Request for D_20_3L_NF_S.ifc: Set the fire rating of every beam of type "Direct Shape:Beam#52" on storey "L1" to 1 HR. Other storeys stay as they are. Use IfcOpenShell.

First a look at what the model holds.

```python
import ifcopenshell
import ifcopenshell.util.element

model = ifcopenshell.open("D_20_3L_NF_S.ifc")
print(model.schema)
storey = next(s for s in model.by_type("IfcBuildingStorey") if s.Name == "L1")
beams = [e for e in ifcopenshell.util.element.get_decomposition(storey) if e.is_a("IfcBeam")]
seen = {}
for e in beams:
    element_type = ifcopenshell.util.element.get_type(e)
    key = (element_type.Name if element_type != e and element_type else None, ifcopenshell.util.element.get_pset(e, "Pset_BeamCommon", "FireRating"))
    seen[key] = seen.get(key, 0) + 1
for (name, value), count in sorted(seen.items(), key=str):
    print(count, "x", name, "|", value)
```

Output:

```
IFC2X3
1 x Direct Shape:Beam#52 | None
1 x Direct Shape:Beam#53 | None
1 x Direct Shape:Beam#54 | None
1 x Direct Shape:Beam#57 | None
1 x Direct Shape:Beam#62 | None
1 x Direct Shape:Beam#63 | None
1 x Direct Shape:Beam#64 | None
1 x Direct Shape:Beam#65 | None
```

```python
import ifcopenshell
import ifcopenshell.api.pset
import ifcopenshell.util.element

model = ifcopenshell.open("D_20_3L_NF_S.ifc")

storey = next(s for s in model.by_type("IfcBuildingStorey") if s.Name == "L1")
beams = [e for e in ifcopenshell.util.element.get_decomposition(storey) if e.is_a("IfcBeam")]

count = 0
for e in beams:
    element_type = ifcopenshell.util.element.get_type(e)
    if element_type in (None, e) or element_type.Name != "Direct Shape:Beam#52":
        continue
    # add_pset returns the element's existing set when there is one.
    pset = ifcopenshell.api.pset.add_pset(model, product=e, name="Pset_BeamCommon")
    ifcopenshell.api.pset.edit_pset(model, pset=pset, properties={"FireRating": "1 HR"})
    count += 1

print(count, "beams updated")

model.write("D_20_3L_NF_S_rev.ifc")
```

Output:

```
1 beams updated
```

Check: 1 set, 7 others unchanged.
